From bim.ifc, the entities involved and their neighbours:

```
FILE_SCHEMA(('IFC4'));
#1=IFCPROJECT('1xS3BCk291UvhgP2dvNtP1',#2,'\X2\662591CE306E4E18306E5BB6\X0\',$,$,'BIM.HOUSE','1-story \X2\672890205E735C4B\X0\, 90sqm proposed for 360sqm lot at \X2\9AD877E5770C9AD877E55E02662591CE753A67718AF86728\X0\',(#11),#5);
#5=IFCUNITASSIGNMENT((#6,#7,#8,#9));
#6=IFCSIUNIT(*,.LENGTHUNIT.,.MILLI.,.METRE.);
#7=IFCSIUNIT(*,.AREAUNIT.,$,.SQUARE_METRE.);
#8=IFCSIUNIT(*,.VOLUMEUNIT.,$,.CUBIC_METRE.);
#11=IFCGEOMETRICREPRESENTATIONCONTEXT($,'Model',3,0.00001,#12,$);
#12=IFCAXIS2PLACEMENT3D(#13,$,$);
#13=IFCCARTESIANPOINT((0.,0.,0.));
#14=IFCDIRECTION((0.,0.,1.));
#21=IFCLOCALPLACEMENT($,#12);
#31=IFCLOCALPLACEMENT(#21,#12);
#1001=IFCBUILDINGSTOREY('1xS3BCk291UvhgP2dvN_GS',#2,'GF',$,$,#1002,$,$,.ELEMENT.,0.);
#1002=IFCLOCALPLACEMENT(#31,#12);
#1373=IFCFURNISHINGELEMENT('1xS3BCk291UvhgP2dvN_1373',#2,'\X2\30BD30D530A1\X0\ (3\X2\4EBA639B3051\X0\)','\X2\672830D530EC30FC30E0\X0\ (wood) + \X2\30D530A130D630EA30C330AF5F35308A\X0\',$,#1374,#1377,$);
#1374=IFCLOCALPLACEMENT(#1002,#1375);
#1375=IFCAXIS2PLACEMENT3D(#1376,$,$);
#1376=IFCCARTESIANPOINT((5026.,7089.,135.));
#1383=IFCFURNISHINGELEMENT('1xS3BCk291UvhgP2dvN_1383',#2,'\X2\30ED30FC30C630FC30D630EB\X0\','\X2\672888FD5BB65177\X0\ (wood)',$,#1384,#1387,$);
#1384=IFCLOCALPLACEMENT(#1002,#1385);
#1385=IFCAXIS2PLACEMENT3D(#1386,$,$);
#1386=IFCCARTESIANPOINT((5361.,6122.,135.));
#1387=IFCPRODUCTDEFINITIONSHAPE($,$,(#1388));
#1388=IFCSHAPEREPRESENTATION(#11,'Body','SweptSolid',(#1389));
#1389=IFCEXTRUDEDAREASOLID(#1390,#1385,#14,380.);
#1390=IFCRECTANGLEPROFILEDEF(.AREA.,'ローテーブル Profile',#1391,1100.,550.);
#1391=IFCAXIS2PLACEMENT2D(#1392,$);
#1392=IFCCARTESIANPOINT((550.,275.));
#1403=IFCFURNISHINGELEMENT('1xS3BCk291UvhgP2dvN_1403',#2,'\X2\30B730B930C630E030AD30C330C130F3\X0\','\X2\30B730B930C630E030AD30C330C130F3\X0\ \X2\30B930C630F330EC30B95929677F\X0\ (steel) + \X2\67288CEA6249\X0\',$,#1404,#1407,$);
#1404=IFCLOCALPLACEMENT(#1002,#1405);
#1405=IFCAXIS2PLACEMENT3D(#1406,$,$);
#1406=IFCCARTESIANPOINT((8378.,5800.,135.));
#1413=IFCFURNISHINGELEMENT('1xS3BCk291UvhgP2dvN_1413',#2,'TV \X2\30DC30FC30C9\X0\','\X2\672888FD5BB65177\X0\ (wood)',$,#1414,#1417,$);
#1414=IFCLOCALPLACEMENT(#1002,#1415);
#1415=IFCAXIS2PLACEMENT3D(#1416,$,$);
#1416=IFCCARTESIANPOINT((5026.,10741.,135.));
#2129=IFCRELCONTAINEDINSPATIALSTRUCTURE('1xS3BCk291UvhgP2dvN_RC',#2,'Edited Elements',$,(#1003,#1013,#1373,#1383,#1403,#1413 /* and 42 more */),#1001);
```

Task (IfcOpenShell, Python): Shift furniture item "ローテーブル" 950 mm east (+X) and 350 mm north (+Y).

```python
import ifcopenshell
import ifcopenshell.api.geometry
import ifcopenshell.util.placement

model = ifcopenshell.open("bim.ifc")

item = model.by_guid("1xS3BCk291UvhgP2dvN_1383")
matrix = ifcopenshell.util.placement.get_local_placement(item.ObjectPlacement)
matrix[0, 3] += 950.0
matrix[1, 3] += 350.0
ifcopenshell.api.geometry.edit_object_placement(model, product=item, matrix=matrix, is_si=False)

print(ifcopenshell.util.placement.get_local_placement(item.ObjectPlacement).round(3) + 0.0)

model.write("bim_edited.ifc")
```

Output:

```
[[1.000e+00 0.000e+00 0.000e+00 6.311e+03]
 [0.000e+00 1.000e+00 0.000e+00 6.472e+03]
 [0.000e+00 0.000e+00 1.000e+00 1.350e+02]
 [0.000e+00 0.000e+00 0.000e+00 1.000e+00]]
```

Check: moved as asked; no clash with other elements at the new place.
